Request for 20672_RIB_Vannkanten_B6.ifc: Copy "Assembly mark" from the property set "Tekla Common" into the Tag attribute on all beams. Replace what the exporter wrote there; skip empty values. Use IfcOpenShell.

First a look at what the model holds.

```python
import ifcopenshell
import ifcopenshell.util.element

model = ifcopenshell.open("20672_RIB_Vannkanten_B6.ifc")
print(model.schema)
beams = model.by_type("IfcBeam")
print(len(beams), "beams")
for e in beams[:8]:
    source = ifcopenshell.util.element.get_pset(e, "Tekla Common", "Assembly mark")
    target = e.Tag
    print(e.id(), repr(source), repr(target), sep=" | ")
```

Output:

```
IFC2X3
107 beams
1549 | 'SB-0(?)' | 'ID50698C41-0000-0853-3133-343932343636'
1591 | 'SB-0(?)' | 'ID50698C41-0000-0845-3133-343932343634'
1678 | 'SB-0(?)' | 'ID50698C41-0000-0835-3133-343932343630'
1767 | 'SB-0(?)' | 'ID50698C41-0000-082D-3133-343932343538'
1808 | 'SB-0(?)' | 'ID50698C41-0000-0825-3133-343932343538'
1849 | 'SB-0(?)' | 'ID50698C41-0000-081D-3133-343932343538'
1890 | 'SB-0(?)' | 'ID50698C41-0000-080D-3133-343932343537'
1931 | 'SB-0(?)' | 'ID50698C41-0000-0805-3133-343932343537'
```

```python
import ifcopenshell
import ifcopenshell.util.element

model = ifcopenshell.open("20672_RIB_Vannkanten_B6.ifc")

count = 0
for e in model.by_type("IfcBeam"):
    value = ifcopenshell.util.element.get_pset(e, "Tekla Common", "Assembly mark")
    current = e.Tag
    if not value or not value.strip() or current == value:
        continue
    e.Tag = value
    count += 1

print(count, "beams updated")

model.write("20672_RIB_Vannkanten_B6-out.ifc")
```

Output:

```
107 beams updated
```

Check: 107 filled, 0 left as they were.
